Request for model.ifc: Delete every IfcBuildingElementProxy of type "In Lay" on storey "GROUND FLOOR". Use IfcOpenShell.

First a look at what the model holds.

```python
import ifcopenshell
import ifcopenshell.util.element

model = ifcopenshell.open("model.ifc")
print(model.schema)
storey = next(s for s in model.by_type("IfcBuildingStorey") if s.Name == "GROUND FLOOR")
proxies = [e for e in ifcopenshell.util.element.get_decomposition(storey) if e.is_a("IfcBuildingElementProxy")]
seen = {}
for e in proxies:
    element_type = ifcopenshell.util.element.get_type(e)
    name = element_type.Name if element_type not in (None, e) else None
    seen[name] = seen.get(name, 0) + 1
for name, count in sorted(seen.items(), key=str):
    print(count, "x", name)
```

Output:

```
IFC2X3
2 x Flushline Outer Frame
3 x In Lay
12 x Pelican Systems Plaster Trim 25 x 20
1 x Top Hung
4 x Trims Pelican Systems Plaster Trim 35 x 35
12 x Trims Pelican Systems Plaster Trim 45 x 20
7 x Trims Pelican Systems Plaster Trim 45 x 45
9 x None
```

```python
import ifcopenshell
import ifcopenshell.api.root
import ifcopenshell.util.element

model = ifcopenshell.open("model.ifc")

storey = next(s for s in model.by_type("IfcBuildingStorey") if s.Name == "GROUND FLOOR")
proxies = [e for e in ifcopenshell.util.element.get_decomposition(storey) if e.is_a("IfcBuildingElementProxy")]
targets = [e for e in proxies if (t := ifcopenshell.util.element.get_type(e)) not in (None, e) and t.Name == "In Lay"]

for e in targets:
    ifcopenshell.api.root.remove_product(model, product=e)
print(len(targets), "removed")

model.write("model_rev.ifc")
```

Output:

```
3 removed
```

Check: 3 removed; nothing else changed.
